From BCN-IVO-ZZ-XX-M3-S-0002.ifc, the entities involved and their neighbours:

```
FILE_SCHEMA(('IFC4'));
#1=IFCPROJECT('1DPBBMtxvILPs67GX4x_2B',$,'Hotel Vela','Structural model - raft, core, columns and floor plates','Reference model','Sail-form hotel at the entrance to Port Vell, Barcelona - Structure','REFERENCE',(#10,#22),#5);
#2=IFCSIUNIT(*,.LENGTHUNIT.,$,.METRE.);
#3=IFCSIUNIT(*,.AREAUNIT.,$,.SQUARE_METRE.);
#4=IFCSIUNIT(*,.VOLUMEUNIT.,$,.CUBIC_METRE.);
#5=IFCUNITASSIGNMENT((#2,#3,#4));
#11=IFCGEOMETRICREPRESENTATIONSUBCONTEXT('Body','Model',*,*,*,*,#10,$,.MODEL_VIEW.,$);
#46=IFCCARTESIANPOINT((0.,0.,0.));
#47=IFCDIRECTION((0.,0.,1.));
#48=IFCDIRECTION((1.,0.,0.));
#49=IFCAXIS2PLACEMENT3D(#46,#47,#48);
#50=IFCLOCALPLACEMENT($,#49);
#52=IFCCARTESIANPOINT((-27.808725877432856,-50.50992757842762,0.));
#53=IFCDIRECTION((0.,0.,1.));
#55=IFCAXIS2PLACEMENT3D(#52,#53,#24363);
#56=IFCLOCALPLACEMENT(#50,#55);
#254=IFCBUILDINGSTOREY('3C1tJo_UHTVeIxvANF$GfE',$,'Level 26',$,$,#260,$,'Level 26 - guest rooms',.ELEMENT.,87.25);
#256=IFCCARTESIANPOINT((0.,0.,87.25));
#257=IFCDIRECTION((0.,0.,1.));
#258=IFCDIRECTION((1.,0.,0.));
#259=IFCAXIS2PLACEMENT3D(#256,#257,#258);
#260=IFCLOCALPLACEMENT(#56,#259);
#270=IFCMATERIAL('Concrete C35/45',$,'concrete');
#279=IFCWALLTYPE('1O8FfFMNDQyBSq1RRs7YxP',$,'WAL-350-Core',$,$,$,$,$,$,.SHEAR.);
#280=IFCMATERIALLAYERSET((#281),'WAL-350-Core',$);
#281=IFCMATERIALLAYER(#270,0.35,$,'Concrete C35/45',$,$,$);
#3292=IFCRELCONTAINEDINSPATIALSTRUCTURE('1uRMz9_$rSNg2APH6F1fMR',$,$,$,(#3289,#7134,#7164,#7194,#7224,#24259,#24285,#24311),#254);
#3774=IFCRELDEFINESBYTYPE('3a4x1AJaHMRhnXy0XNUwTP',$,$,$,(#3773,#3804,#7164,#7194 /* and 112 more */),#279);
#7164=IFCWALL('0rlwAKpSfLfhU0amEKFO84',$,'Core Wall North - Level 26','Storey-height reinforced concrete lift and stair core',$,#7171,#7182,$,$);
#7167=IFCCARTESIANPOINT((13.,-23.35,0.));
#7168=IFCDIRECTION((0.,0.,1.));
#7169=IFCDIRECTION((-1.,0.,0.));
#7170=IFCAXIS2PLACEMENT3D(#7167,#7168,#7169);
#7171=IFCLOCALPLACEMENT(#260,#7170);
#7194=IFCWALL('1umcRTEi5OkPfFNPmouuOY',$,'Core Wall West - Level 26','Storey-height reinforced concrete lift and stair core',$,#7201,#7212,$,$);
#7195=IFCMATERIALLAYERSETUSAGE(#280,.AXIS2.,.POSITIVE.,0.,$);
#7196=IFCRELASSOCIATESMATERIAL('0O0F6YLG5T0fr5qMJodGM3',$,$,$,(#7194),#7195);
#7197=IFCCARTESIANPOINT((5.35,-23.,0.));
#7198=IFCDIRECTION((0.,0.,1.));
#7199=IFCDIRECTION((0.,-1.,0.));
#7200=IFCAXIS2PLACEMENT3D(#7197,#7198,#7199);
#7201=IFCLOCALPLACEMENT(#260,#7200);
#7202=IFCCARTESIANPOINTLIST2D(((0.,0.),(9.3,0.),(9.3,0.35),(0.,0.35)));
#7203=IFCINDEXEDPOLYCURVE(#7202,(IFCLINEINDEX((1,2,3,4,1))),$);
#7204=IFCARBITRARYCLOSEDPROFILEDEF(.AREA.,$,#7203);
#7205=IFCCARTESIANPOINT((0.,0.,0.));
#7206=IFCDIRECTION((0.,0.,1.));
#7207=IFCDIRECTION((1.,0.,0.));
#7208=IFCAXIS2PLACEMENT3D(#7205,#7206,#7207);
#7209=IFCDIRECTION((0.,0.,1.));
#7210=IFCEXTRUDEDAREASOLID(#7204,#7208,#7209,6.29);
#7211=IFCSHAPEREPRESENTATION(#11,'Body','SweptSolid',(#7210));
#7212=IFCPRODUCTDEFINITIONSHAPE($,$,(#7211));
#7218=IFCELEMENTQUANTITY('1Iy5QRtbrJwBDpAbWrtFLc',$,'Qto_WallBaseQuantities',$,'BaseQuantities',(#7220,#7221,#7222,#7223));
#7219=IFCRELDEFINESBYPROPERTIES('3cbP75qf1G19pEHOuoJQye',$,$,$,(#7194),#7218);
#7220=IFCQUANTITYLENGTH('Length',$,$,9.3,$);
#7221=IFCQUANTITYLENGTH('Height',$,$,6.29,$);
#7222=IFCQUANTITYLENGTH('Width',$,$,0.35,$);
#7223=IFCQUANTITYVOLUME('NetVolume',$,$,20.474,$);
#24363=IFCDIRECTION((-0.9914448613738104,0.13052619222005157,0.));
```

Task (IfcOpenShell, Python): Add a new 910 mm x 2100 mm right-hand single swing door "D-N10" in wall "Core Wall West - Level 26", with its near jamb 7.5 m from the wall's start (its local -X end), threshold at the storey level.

```python
import numpy as np
import ifcopenshell
import ifcopenshell.api.feature
import ifcopenshell.api.geometry
import ifcopenshell.api.pset
import ifcopenshell.api.root
import ifcopenshell.api.spatial
import ifcopenshell.geom
import ifcopenshell.util.element
import ifcopenshell.util.placement
import ifcopenshell.util.representation
import ifcopenshell.util.shape
import ifcopenshell.util.unit

model = ifcopenshell.open("BCN-IVO-ZZ-XX-M3-S-0002.ifc")
unit_scale = ifcopenshell.util.unit.calculate_unit_scale(model)
volume_scale = ifcopenshell.util.unit.calculate_unit_scale(model, "VOLUMEUNIT")
settings = ifcopenshell.geom.settings()


def volume(element):
    """Net volume in cubic metres, openings subtracted."""
    shape = ifcopenshell.geom.create_shape(settings, element)
    return ifcopenshell.util.shape.get_volume(shape.geometry)


wall = model.by_guid("1umcRTEi5OkPfFNPmouuOY")
storey = ifcopenshell.util.element.get_container(wall, ifc_class="IfcBuildingStorey")
context = ifcopenshell.util.representation.get_context(model, "Model", "Body", "MODEL_VIEW")
before = volume(wall)

width, height, from_end, sill = 0.91, 2.1, 7.5, 0.0  # metres

# The wall runs along its own X axis, and the end named is its -X end.
wall_shape = ifcopenshell.geom.create_shape(settings, wall)
x, y, z = ifcopenshell.util.shape.get_vertices(wall_shape.geometry).T
start = x.min() + from_end
face, thickness = float(y.min()), float(y.max() - y.min())
wall_matrix = ifcopenshell.util.placement.get_local_placement(wall.ObjectPlacement)
level = ifcopenshell.util.placement.get_local_placement(storey.ObjectPlacement)[2, 3]


def in_wall(x, y):
    """Placement at x, y metres in the wall's axes, at sill height."""
    matrix = wall_matrix.copy()
    matrix[:, 3] = wall_matrix @ np.array([x / unit_scale, y / unit_scale, 0.0, 1.0])
    matrix[2, 3] = level + sill / unit_scale
    return matrix


# Opening: a box that overshoots both wall faces by 50 mm.
opening = ifcopenshell.api.root.create_entity(model, ifc_class="IfcOpeningElement", predefined_type="OPENING")
box = ifcopenshell.api.geometry.add_wall_representation(
    model, context=context, length=width, height=height, thickness=thickness + 0.1
)
ifcopenshell.api.geometry.assign_representation(model, product=opening, representation=box)
ifcopenshell.api.geometry.edit_object_placement(model, product=opening, matrix=in_wall(start, face - 0.05), is_si=False)
ifcopenshell.api.feature.add_feature(model, feature=opening, element=wall)

door = ifcopenshell.api.root.create_entity(model, ifc_class="IfcDoor", name="D-N10", predefined_type="DOOR")
door.OverallWidth, door.OverallHeight = width / unit_scale, height / unit_scale
door.OperationType = "SINGLE_SWING_RIGHT"
body = ifcopenshell.api.geometry.add_door_representation(
    model,
    context=context,
    overall_width=door.OverallWidth,
    overall_height=door.OverallHeight,
    operation_type="SINGLE_SWING_RIGHT",
    lining_properties={"LiningDepth": thickness / unit_scale, "ThresholdDepth": thickness / unit_scale},
)
ifcopenshell.api.geometry.assign_representation(model, product=door, representation=body)
ifcopenshell.api.spatial.assign_container(model, products=[door], relating_structure=storey)
ifcopenshell.api.feature.add_filling(model, opening=opening, element=door)

# The lining spans the wall, so the door starts at the wall face.
ifcopenshell.api.geometry.edit_object_placement(model, product=door, matrix=in_wall(start, face), is_si=False)

after = volume(wall)

# Update the wall's stored quantities.
qto = model.by_id(ifcopenshell.util.element.get_pset(wall, "Qto_WallBaseQuantities", should_inherit=False)["id"])
ifcopenshell.api.pset.edit_qto(model, qto=qto, properties={"NetVolume": after / volume_scale})

print(f"wall volume {before:.3f} -> {after:.3f} m3")

model.write("BCN-IVO-ZZ-XX-M3-S-0002_updated.ifc")
```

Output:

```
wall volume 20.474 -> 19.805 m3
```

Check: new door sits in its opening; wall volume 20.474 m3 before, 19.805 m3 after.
